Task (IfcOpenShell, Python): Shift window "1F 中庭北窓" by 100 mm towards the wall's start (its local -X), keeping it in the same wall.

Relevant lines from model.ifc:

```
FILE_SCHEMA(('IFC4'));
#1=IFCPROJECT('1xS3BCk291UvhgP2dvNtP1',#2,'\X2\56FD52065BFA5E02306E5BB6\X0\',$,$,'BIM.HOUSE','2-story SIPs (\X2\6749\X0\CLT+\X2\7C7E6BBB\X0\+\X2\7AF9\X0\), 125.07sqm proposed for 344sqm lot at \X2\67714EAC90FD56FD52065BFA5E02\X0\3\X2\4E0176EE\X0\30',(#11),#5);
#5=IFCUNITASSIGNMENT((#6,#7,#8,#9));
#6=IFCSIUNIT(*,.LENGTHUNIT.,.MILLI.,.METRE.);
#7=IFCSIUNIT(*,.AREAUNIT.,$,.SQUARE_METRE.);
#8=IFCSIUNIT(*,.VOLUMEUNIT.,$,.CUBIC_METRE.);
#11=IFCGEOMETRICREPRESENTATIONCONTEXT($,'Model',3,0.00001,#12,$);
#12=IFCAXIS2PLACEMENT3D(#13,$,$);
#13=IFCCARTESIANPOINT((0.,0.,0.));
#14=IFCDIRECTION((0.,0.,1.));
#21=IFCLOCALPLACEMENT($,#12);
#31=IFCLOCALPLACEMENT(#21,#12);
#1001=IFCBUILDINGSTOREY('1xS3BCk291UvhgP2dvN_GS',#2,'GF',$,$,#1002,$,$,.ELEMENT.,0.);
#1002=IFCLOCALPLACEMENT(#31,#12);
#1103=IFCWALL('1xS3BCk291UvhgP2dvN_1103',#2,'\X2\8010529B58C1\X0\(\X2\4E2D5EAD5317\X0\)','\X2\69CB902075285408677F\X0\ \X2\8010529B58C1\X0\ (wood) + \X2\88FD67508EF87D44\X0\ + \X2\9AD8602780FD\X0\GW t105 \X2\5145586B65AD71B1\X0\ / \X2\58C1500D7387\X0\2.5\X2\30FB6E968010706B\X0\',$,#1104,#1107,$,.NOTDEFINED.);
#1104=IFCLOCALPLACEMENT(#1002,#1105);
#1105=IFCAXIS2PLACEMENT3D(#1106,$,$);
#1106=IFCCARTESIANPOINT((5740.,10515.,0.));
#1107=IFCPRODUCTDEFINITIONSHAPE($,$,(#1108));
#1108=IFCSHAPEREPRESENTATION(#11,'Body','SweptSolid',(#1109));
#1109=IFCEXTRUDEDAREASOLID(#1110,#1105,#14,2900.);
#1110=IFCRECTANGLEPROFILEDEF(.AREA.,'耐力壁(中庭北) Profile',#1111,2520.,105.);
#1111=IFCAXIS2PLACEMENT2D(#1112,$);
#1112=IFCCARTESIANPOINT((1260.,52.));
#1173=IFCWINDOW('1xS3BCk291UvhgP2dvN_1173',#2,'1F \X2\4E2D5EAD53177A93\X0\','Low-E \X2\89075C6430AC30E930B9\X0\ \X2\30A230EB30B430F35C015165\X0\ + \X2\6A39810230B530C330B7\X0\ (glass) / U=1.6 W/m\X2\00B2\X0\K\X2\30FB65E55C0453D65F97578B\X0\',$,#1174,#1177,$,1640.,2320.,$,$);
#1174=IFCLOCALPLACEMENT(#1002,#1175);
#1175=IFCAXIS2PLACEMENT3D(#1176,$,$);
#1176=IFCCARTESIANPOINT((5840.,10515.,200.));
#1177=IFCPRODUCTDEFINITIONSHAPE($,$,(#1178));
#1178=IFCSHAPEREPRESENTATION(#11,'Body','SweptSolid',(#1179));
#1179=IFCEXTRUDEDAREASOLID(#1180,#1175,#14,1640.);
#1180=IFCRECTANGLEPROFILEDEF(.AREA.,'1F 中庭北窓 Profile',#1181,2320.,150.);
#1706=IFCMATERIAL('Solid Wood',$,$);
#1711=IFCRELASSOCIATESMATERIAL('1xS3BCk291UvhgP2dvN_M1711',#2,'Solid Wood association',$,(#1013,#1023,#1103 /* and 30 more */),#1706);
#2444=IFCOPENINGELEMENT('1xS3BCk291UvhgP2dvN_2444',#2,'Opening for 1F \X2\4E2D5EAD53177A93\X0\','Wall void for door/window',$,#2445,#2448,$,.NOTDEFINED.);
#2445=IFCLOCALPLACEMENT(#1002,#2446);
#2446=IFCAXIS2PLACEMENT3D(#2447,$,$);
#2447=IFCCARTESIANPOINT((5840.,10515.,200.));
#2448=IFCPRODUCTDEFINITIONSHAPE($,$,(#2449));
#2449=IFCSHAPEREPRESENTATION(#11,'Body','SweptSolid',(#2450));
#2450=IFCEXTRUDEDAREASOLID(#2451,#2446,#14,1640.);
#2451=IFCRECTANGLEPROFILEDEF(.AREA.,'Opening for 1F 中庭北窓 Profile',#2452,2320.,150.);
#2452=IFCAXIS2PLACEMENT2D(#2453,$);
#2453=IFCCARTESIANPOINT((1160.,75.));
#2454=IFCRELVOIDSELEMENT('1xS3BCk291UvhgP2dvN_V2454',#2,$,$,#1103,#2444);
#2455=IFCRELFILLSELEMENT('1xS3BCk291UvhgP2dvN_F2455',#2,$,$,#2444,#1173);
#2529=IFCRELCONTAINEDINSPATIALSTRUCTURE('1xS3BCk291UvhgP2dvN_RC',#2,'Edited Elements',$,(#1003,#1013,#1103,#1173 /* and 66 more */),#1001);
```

```python
import ifcopenshell
import ifcopenshell.api.geometry
import ifcopenshell.util.placement
import ifcopenshell.util.unit

model = ifcopenshell.open("model.ifc")
unit_scale = ifcopenshell.util.unit.calculate_unit_scale(model)

window = model.by_guid("1xS3BCk291UvhgP2dvN_1173")
opening = window.FillsVoids[0].RelatingOpeningElement
wall = opening.VoidsElements[0].RelatingBuildingElement

wall_matrix = ifcopenshell.util.placement.get_local_placement(wall.ObjectPlacement)
shift = wall_matrix[:3, 0] * -0.1 / unit_scale
before = ifcopenshell.util.placement.get_local_placement(window.ObjectPlacement)[:3, 3].copy()

# The window is not placed relative to its opening, so move both.
for product in (opening, window):
    matrix = ifcopenshell.util.placement.get_local_placement(product.ObjectPlacement)
    matrix[:3, 3] += shift
    ifcopenshell.api.geometry.edit_object_placement(model, product=product, matrix=matrix, is_si=False)

after = ifcopenshell.util.placement.get_local_placement(window.ObjectPlacement)[:3, 3]
print("window moved by", (after - before).round(3) + 0.0)

model.write("model_rev.ifc")
```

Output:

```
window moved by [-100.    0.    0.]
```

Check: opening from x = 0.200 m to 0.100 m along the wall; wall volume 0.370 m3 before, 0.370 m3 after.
